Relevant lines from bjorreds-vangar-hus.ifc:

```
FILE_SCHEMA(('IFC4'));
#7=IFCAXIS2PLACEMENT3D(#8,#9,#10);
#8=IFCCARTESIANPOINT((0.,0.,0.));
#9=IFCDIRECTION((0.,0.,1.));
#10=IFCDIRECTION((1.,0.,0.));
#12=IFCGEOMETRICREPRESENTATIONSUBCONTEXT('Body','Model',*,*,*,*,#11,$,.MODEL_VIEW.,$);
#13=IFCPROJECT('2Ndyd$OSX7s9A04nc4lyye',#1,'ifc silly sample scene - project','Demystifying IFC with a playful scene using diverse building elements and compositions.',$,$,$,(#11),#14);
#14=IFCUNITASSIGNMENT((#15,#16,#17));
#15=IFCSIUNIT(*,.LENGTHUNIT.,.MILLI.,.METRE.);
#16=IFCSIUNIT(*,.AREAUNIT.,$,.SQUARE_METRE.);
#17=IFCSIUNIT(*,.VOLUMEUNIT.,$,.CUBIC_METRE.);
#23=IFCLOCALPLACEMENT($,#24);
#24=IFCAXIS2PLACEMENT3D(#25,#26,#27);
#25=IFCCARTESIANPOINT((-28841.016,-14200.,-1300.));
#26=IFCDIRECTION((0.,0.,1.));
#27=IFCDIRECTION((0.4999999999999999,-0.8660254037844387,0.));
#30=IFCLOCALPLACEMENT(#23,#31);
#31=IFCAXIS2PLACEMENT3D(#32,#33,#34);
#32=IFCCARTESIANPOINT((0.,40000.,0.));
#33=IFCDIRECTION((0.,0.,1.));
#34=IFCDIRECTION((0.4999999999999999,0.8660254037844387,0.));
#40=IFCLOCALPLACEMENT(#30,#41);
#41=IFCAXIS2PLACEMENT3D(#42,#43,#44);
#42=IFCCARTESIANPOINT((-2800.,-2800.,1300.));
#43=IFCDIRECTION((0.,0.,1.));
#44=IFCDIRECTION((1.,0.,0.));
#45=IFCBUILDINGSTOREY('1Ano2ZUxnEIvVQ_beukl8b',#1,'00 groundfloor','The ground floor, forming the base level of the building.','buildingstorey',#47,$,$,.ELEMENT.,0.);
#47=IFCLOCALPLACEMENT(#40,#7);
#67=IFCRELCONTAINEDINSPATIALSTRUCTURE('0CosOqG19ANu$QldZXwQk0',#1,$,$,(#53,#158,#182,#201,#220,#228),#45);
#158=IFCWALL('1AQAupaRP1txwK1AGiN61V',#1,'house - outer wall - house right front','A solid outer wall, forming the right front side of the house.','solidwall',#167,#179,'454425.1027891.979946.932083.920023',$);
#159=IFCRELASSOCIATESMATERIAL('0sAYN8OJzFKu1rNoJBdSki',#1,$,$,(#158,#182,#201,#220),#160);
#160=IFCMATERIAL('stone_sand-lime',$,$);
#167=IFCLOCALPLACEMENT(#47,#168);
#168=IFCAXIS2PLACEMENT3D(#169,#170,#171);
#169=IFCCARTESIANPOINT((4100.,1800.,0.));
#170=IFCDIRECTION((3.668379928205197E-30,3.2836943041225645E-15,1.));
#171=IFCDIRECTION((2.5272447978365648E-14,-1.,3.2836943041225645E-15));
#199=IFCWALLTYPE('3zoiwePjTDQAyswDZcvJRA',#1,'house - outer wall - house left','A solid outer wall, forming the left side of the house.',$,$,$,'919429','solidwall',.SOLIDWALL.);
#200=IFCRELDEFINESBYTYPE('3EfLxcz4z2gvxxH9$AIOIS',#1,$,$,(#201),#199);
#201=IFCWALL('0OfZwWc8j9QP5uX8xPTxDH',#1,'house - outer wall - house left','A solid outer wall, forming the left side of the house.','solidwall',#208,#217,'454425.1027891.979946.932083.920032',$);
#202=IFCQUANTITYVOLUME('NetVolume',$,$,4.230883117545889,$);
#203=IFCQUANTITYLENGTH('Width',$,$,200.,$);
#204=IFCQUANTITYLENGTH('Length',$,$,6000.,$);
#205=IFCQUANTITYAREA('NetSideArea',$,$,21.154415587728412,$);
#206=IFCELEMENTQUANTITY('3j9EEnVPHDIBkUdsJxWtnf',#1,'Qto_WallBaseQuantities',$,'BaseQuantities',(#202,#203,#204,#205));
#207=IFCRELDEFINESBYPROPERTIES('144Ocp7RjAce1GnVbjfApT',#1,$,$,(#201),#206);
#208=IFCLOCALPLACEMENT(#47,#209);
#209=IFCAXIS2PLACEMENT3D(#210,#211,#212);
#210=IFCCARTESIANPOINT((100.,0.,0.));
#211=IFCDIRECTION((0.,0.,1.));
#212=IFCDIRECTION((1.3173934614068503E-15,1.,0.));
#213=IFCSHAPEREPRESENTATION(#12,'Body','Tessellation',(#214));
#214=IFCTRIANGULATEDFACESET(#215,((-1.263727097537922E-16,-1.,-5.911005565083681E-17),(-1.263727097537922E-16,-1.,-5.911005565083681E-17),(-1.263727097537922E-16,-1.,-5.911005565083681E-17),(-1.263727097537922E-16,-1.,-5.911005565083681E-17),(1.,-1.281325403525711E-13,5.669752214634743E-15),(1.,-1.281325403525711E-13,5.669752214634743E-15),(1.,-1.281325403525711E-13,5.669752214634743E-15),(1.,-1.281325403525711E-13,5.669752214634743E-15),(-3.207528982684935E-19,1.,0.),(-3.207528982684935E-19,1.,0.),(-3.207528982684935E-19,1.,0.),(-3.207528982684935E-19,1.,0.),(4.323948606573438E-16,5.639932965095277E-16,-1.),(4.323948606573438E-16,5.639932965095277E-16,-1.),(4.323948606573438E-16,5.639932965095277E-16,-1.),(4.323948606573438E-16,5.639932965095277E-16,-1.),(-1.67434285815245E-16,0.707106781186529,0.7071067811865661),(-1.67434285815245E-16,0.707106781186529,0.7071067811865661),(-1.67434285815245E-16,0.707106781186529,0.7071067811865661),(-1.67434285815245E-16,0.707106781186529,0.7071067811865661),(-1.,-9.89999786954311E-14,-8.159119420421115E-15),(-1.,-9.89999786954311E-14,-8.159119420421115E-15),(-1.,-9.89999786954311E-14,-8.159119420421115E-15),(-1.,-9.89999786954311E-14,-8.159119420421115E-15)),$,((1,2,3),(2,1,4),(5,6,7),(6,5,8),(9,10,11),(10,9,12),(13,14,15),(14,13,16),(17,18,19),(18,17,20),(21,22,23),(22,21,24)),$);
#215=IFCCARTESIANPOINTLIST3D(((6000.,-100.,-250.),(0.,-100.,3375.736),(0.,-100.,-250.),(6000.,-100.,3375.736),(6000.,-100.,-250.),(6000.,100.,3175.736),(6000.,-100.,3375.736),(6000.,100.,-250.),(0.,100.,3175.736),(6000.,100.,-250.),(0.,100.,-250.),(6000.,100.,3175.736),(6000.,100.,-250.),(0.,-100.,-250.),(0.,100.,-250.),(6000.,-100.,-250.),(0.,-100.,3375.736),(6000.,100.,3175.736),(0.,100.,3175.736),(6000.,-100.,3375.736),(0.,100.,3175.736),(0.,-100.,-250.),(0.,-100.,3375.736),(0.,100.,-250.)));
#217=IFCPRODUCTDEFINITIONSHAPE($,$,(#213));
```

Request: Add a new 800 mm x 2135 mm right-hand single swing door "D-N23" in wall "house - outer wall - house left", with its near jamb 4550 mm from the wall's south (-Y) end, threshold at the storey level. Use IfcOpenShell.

```python
import numpy as np
import ifcopenshell
import ifcopenshell.api.feature
import ifcopenshell.api.geometry
import ifcopenshell.api.pset
import ifcopenshell.api.root
import ifcopenshell.api.spatial
import ifcopenshell.geom
import ifcopenshell.util.element
import ifcopenshell.util.placement
import ifcopenshell.util.representation
import ifcopenshell.util.shape
import ifcopenshell.util.unit

model = ifcopenshell.open("bjorreds-vangar-hus.ifc")
unit_scale = ifcopenshell.util.unit.calculate_unit_scale(model)
area_scale = ifcopenshell.util.unit.calculate_unit_scale(model, "AREAUNIT")
volume_scale = ifcopenshell.util.unit.calculate_unit_scale(model, "VOLUMEUNIT")
settings = ifcopenshell.geom.settings()


def volume(element):
    """Net volume in cubic metres, openings subtracted."""
    shape = ifcopenshell.geom.create_shape(settings, element)
    return ifcopenshell.util.shape.get_volume(shape.geometry)


wall = model.by_id(201)
storey = ifcopenshell.util.element.get_container(wall, ifc_class="IfcBuildingStorey")
context = ifcopenshell.util.representation.get_context(model, "Model", "Body", "MODEL_VIEW")
before = volume(wall)

width, height, from_end, sill = 0.8, 2.135, 4.55, 0.0  # metres

# The wall runs along its own X axis, and the end named is its -X end.
wall_shape = ifcopenshell.geom.create_shape(settings, wall)
x, y, z = ifcopenshell.util.shape.get_vertices(wall_shape.geometry).T
start = x.min() + from_end
face, thickness = float(y.min()), float(y.max() - y.min())
wall_matrix = ifcopenshell.util.placement.get_local_placement(wall.ObjectPlacement)
level = ifcopenshell.util.placement.get_local_placement(storey.ObjectPlacement)[2, 3]


def in_wall(x, y):
    """Placement at x, y metres in the wall's axes, at sill height."""
    matrix = wall_matrix.copy()
    matrix[:, 3] = wall_matrix @ np.array([x / unit_scale, y / unit_scale, 0.0, 1.0])
    matrix[2, 3] = level + sill / unit_scale
    return matrix


# Opening: a box that overshoots both wall faces by 50 mm.
opening = ifcopenshell.api.root.create_entity(model, ifc_class="IfcOpeningElement", predefined_type="OPENING")
box = ifcopenshell.api.geometry.add_wall_representation(
    model, context=context, length=width, height=height, thickness=thickness + 0.1
)
ifcopenshell.api.geometry.assign_representation(model, product=opening, representation=box)
ifcopenshell.api.geometry.edit_object_placement(model, product=opening, matrix=in_wall(start, face - 0.05), is_si=False)
ifcopenshell.api.feature.add_feature(model, feature=opening, element=wall)

door = ifcopenshell.api.root.create_entity(model, ifc_class="IfcDoor", name="D-N23", predefined_type="DOOR")
door.OverallWidth, door.OverallHeight = width / unit_scale, height / unit_scale
door.OperationType = "SINGLE_SWING_RIGHT"
body = ifcopenshell.api.geometry.add_door_representation(
    model,
    context=context,
    overall_width=door.OverallWidth,
    overall_height=door.OverallHeight,
    operation_type="SINGLE_SWING_RIGHT",
    lining_properties={"LiningDepth": thickness / unit_scale, "ThresholdDepth": thickness / unit_scale},
)
ifcopenshell.api.geometry.assign_representation(model, product=door, representation=body)
ifcopenshell.api.spatial.assign_container(model, products=[door], relating_structure=storey)
ifcopenshell.api.feature.add_filling(model, opening=opening, element=door)

# The lining spans the wall, so the door starts at the wall face.
ifcopenshell.api.geometry.edit_object_placement(model, product=door, matrix=in_wall(start, face), is_si=False)

after = volume(wall)

# Update the wall's stored quantities.
qto = model.by_id(ifcopenshell.util.element.get_pset(wall, "Qto_WallBaseQuantities", should_inherit=False)["id"])
ifcopenshell.api.pset.edit_qto(model, qto=qto, properties={
    "NetVolume": after / volume_scale,
    "NetSideArea": after / thickness / area_scale,
})

print(f"wall volume {before:.3f} -> {after:.3f} m3")

model.write("bjorreds-vangar-hus_updated.ifc")
```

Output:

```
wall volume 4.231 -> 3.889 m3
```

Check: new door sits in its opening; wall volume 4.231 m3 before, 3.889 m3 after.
